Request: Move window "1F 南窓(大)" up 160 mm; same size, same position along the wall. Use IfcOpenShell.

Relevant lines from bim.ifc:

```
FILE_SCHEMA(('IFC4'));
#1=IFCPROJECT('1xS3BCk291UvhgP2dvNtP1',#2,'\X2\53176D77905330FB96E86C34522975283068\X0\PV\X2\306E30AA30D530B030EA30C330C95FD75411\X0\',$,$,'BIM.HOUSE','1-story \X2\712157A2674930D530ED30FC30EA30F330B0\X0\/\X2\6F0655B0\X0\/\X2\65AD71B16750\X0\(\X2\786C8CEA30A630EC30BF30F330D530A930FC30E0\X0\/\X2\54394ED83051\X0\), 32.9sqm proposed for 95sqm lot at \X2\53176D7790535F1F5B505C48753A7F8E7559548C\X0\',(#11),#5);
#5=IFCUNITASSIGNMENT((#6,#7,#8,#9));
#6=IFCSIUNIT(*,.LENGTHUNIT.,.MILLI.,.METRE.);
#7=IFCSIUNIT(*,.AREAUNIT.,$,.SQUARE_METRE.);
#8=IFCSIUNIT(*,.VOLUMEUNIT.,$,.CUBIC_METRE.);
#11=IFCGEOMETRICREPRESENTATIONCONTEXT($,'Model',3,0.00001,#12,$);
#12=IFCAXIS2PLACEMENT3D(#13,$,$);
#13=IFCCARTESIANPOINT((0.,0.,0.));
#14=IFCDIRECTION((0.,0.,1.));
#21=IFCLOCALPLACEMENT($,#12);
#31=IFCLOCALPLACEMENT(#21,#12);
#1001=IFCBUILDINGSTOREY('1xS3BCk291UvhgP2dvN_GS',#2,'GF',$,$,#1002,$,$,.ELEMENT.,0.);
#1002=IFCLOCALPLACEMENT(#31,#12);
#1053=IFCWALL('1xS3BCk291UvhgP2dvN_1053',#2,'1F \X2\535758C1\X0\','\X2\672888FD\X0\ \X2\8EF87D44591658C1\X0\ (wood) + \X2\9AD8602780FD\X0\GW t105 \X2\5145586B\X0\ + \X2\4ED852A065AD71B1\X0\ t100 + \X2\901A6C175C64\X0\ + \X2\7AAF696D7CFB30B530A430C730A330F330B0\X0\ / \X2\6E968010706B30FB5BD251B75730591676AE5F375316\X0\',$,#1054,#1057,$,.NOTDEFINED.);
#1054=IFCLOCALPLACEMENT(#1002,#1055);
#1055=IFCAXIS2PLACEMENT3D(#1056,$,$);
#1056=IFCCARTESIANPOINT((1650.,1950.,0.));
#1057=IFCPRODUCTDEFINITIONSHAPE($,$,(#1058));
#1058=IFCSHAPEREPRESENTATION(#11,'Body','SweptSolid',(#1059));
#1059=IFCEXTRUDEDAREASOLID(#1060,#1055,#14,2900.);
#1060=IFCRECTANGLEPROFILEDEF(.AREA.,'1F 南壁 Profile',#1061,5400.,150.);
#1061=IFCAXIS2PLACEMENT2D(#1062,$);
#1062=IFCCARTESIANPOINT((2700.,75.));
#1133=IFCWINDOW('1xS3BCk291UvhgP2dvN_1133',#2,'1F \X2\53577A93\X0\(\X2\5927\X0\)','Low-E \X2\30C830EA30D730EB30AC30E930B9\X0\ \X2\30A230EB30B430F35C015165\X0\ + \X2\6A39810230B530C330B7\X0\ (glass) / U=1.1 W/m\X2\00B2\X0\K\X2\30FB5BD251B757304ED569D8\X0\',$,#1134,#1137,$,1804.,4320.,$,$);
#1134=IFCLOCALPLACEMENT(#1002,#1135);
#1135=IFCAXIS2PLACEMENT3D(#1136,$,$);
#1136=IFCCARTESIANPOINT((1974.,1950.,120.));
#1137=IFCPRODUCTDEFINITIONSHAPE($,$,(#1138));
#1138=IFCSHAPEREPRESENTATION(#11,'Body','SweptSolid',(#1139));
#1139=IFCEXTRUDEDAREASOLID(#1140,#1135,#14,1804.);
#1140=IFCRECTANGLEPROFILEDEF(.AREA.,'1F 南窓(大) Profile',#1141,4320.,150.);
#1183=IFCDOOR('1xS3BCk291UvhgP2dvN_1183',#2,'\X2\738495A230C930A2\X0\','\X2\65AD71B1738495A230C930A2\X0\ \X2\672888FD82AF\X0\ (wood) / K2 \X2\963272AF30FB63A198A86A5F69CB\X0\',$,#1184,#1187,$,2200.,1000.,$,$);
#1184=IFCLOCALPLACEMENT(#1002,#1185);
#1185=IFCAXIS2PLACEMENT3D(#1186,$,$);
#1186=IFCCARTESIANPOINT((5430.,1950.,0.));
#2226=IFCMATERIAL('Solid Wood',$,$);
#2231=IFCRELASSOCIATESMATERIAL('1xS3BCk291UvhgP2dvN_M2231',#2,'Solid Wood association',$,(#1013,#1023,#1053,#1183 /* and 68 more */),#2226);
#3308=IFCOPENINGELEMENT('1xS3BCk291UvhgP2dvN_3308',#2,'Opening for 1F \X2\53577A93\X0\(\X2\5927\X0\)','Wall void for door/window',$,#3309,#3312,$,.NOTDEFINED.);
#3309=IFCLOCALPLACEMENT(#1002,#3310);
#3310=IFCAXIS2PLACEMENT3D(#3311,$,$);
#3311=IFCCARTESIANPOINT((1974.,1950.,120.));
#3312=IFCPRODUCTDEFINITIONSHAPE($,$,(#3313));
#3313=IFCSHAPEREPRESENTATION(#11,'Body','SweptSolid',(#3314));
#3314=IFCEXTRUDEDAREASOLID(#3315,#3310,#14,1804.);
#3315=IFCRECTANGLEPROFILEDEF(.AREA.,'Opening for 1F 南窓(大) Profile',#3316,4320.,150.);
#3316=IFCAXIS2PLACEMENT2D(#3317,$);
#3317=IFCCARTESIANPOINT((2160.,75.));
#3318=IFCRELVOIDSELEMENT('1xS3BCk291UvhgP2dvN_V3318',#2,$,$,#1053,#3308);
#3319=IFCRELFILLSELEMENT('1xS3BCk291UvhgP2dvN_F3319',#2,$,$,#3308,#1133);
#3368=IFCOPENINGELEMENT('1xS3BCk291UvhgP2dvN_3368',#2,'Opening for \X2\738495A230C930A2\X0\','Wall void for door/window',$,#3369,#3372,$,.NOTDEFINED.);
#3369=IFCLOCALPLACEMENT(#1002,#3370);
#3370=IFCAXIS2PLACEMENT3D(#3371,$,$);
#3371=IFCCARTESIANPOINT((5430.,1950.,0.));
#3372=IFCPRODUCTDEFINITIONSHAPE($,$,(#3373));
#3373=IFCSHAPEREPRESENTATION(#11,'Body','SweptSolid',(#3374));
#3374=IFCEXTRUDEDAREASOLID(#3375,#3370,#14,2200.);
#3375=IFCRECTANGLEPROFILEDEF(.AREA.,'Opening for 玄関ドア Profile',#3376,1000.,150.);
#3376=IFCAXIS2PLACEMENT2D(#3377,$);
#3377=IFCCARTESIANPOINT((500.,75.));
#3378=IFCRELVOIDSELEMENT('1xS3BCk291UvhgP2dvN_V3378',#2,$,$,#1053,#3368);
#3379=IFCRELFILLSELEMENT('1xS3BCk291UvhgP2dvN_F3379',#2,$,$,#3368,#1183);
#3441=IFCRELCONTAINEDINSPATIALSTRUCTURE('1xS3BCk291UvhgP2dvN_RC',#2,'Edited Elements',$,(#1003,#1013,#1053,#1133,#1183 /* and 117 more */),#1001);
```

```python
import numpy as np
import ifcopenshell
import ifcopenshell.api.geometry
import ifcopenshell.util.placement
import ifcopenshell.util.unit

model = ifcopenshell.open("bim.ifc")
unit_scale = ifcopenshell.util.unit.calculate_unit_scale(model)

window = model.by_guid("1xS3BCk291UvhgP2dvN_1133")
opening = window.FillsVoids[0].RelatingOpeningElement
dz = 0.16 / unit_scale

shift = np.array([0.0, 0.0, dz])
# The window is not placed relative to its opening, so move both.
for product in (opening, window):
    matrix = ifcopenshell.util.placement.get_local_placement(product.ObjectPlacement)
    matrix[:3, 3] += shift
    ifcopenshell.api.geometry.edit_object_placement(model, product=product, matrix=matrix, is_si=False)

print(f"moved by {dz * unit_scale:+.3f} m")

model.write("bim_updated.ifc")
```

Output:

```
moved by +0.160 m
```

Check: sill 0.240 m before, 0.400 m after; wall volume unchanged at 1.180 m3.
